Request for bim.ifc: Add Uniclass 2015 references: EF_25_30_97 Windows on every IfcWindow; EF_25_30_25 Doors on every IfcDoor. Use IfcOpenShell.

First a look at what the model holds.

```python
import ifcopenshell

model = ifcopenshell.open("bim.ifc")
print(model.schema)
print("classifications:", [c.Name for c in model.by_type("IfcClassification")])
for ifc_class in ("IfcDoor", "IfcRoof", "IfcStair", "IfcWall", "IfcWindow"):
    print(ifc_class, len(model.by_type(ifc_class)))
```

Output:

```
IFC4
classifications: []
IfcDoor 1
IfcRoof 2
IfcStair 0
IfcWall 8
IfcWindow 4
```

```python
import ifcopenshell
import ifcopenshell.api.classification

model = ifcopenshell.open("bim.ifc")

system = ifcopenshell.api.classification.add_classification(model, classification="Uniclass 2015")

codes = {
    "IfcWindow": ("EF_25_30_97", "Windows"),
    "IfcDoor": ("EF_25_30_25", "Doors"),
}
for ifc_class, (code, name) in codes.items():
    products = model.by_type(ifc_class)
    ifcopenshell.api.classification.add_reference(
        model, products=products, classification=system, identification=code, name=name
    )
    print(code, len(products))

model.write("bim_v2.ifc")
```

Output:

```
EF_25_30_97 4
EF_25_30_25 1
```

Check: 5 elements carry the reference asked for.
